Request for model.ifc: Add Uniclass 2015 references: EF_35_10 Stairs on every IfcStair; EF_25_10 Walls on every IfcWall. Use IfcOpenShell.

First a look at what the model holds.

```python
import ifcopenshell

model = ifcopenshell.open("model.ifc")
print(model.schema)
print("classifications:", [c.Name for c in model.by_type("IfcClassification")])
for ifc_class in ("IfcDoor", "IfcRoof", "IfcStair", "IfcWall", "IfcWindow"):
    print(ifc_class, len(model.by_type(ifc_class)))
```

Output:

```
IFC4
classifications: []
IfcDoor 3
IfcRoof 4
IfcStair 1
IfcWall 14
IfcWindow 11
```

```python
import ifcopenshell
import ifcopenshell.api.classification

model = ifcopenshell.open("model.ifc")

system = ifcopenshell.api.classification.add_classification(model, classification="Uniclass 2015")

codes = {
    "IfcStair": ("EF_35_10", "Stairs"),
    "IfcWall": ("EF_25_10", "Walls"),
}
for ifc_class, (code, name) in codes.items():
    products = model.by_type(ifc_class)
    ifcopenshell.api.classification.add_reference(
        model, products=products, classification=system, identification=code, name=name
    )
    print(code, len(products))

model.write("model-out.ifc")
```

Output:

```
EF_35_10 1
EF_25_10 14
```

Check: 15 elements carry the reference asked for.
